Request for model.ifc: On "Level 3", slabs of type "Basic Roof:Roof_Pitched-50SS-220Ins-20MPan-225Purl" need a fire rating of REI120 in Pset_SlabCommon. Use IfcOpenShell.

First a look at what the model holds.

```python
import ifcopenshell
import ifcopenshell.util.element

model = ifcopenshell.open("model.ifc")
print(model.schema)
storey = next(s for s in model.by_type("IfcBuildingStorey") if s.Name == "Level 3")
slabs = [e for e in ifcopenshell.util.element.get_decomposition(storey) if e.is_a("IfcSlab")]
seen = {}
for e in slabs:
    element_type = ifcopenshell.util.element.get_type(e)
    key = (element_type.Name if element_type != e and element_type else None, ifcopenshell.util.element.get_pset(e, "Pset_SlabCommon", "FireRating"))
    seen[key] = seen.get(key, 0) + 1
for (name, value), count in sorted(seen.items(), key=str):
    print(count, "x", name, "|", value)
```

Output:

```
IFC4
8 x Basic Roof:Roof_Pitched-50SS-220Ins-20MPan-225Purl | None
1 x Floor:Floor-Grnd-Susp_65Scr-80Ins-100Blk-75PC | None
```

```python
import ifcopenshell
import ifcopenshell.api.pset
import ifcopenshell.util.element

model = ifcopenshell.open("model.ifc")

storey = next(s for s in model.by_type("IfcBuildingStorey") if s.Name == "Level 3")
slabs = [e for e in ifcopenshell.util.element.get_decomposition(storey) if e.is_a("IfcSlab")]

count = 0
for e in slabs:
    element_type = ifcopenshell.util.element.get_type(e)
    if element_type in (None, e) or element_type.Name != "Basic Roof:Roof_Pitched-50SS-220Ins-20MPan-225Purl":
        continue
    # add_pset returns the element's existing set when there is one.
    pset = ifcopenshell.api.pset.add_pset(model, product=e, name="Pset_SlabCommon")
    ifcopenshell.api.pset.edit_pset(model, pset=pset, properties={"FireRating": "REI120"})
    count += 1

print(count, "slabs updated")

model.write("model_rev.ifc")
```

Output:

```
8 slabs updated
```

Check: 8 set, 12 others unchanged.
